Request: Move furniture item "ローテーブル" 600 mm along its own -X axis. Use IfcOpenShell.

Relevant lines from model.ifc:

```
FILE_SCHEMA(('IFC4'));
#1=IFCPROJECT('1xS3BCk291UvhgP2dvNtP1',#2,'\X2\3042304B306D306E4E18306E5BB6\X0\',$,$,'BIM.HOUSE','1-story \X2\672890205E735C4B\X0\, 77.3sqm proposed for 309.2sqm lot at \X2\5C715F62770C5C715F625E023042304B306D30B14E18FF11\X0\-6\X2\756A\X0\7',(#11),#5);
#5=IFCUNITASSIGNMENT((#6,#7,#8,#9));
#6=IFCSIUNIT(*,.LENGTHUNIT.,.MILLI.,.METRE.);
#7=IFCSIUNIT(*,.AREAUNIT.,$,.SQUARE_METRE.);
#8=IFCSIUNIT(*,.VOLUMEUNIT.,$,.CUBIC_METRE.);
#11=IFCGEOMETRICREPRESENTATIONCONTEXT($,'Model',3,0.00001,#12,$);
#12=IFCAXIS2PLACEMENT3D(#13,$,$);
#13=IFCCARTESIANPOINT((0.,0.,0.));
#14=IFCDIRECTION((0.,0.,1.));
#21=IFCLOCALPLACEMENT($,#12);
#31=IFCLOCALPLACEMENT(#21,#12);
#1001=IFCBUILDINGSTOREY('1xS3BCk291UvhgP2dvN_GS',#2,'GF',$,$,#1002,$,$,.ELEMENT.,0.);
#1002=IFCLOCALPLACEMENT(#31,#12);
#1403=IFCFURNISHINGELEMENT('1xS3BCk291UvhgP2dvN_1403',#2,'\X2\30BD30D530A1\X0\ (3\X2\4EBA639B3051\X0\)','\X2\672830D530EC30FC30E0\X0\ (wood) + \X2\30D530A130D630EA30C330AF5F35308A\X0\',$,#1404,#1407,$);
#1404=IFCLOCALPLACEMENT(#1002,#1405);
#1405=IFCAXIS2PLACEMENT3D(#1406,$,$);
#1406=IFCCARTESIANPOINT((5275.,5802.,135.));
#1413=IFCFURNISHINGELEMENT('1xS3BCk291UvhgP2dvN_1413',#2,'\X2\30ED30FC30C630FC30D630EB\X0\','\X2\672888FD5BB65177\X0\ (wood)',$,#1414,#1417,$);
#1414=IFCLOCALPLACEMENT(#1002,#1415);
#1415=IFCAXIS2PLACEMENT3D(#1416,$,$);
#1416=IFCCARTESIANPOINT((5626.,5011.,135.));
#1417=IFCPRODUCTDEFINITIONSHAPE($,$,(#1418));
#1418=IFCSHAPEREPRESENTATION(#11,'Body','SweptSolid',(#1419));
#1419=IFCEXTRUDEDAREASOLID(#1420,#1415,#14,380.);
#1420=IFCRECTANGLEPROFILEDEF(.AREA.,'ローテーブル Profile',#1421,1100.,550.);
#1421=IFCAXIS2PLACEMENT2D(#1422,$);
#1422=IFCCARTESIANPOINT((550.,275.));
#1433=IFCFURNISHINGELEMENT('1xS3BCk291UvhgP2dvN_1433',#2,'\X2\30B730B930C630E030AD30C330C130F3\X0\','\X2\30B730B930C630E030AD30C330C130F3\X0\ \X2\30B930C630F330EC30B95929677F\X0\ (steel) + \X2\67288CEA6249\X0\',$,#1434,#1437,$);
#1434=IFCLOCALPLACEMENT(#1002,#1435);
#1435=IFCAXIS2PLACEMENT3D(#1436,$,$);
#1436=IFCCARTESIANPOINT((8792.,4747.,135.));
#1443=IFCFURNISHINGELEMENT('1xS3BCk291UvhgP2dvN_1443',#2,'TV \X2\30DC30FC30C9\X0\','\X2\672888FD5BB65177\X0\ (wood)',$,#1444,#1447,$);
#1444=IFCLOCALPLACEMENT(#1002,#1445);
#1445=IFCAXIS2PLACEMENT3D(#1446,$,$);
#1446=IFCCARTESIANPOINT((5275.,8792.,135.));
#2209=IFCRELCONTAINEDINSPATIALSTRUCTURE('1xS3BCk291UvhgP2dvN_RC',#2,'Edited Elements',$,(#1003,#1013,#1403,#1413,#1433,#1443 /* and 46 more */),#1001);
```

```python
import ifcopenshell
import ifcopenshell.api.geometry
import ifcopenshell.util.placement

model = ifcopenshell.open("model.ifc")

item = model.by_guid("1xS3BCk291UvhgP2dvN_1413")
matrix = ifcopenshell.util.placement.get_local_placement(item.ObjectPlacement)
matrix[:3, 3] -= matrix[:3, 0] * 600.0
ifcopenshell.api.geometry.edit_object_placement(model, product=item, matrix=matrix, is_si=False)

print(ifcopenshell.util.placement.get_local_placement(item.ObjectPlacement).round(3) + 0.0)

model.write("model-out.ifc")
```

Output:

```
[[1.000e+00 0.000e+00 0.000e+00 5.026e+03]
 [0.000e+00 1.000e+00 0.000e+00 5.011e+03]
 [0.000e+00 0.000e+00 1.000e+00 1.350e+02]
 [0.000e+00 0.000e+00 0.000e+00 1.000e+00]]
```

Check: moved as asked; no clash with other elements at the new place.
